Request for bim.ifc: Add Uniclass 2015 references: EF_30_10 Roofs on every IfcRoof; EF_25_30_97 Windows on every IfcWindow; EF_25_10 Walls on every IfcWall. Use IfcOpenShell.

First a look at what the model holds.

```python
import ifcopenshell

model = ifcopenshell.open("bim.ifc")
print(model.schema)
print("classifications:", [c.Name for c in model.by_type("IfcClassification")])
for ifc_class in ("IfcDoor", "IfcRoof", "IfcStair", "IfcWall", "IfcWindow"):
    print(ifc_class, len(model.by_type(ifc_class)))
```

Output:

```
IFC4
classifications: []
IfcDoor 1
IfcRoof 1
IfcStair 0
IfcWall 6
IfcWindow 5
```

```python
import ifcopenshell
import ifcopenshell.api.classification

model = ifcopenshell.open("bim.ifc")

system = ifcopenshell.api.classification.add_classification(model, classification="Uniclass 2015")

codes = {
    "IfcRoof": ("EF_30_10", "Roofs"),
    "IfcWindow": ("EF_25_30_97", "Windows"),
    "IfcWall": ("EF_25_10", "Walls"),
}
for ifc_class, (code, name) in codes.items():
    products = model.by_type(ifc_class)
    ifcopenshell.api.classification.add_reference(
        model, products=products, classification=system, identification=code, name=name
    )
    print(code, len(products))

model.write("bim_v2.ifc")
```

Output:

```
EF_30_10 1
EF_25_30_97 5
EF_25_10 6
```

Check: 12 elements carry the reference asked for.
